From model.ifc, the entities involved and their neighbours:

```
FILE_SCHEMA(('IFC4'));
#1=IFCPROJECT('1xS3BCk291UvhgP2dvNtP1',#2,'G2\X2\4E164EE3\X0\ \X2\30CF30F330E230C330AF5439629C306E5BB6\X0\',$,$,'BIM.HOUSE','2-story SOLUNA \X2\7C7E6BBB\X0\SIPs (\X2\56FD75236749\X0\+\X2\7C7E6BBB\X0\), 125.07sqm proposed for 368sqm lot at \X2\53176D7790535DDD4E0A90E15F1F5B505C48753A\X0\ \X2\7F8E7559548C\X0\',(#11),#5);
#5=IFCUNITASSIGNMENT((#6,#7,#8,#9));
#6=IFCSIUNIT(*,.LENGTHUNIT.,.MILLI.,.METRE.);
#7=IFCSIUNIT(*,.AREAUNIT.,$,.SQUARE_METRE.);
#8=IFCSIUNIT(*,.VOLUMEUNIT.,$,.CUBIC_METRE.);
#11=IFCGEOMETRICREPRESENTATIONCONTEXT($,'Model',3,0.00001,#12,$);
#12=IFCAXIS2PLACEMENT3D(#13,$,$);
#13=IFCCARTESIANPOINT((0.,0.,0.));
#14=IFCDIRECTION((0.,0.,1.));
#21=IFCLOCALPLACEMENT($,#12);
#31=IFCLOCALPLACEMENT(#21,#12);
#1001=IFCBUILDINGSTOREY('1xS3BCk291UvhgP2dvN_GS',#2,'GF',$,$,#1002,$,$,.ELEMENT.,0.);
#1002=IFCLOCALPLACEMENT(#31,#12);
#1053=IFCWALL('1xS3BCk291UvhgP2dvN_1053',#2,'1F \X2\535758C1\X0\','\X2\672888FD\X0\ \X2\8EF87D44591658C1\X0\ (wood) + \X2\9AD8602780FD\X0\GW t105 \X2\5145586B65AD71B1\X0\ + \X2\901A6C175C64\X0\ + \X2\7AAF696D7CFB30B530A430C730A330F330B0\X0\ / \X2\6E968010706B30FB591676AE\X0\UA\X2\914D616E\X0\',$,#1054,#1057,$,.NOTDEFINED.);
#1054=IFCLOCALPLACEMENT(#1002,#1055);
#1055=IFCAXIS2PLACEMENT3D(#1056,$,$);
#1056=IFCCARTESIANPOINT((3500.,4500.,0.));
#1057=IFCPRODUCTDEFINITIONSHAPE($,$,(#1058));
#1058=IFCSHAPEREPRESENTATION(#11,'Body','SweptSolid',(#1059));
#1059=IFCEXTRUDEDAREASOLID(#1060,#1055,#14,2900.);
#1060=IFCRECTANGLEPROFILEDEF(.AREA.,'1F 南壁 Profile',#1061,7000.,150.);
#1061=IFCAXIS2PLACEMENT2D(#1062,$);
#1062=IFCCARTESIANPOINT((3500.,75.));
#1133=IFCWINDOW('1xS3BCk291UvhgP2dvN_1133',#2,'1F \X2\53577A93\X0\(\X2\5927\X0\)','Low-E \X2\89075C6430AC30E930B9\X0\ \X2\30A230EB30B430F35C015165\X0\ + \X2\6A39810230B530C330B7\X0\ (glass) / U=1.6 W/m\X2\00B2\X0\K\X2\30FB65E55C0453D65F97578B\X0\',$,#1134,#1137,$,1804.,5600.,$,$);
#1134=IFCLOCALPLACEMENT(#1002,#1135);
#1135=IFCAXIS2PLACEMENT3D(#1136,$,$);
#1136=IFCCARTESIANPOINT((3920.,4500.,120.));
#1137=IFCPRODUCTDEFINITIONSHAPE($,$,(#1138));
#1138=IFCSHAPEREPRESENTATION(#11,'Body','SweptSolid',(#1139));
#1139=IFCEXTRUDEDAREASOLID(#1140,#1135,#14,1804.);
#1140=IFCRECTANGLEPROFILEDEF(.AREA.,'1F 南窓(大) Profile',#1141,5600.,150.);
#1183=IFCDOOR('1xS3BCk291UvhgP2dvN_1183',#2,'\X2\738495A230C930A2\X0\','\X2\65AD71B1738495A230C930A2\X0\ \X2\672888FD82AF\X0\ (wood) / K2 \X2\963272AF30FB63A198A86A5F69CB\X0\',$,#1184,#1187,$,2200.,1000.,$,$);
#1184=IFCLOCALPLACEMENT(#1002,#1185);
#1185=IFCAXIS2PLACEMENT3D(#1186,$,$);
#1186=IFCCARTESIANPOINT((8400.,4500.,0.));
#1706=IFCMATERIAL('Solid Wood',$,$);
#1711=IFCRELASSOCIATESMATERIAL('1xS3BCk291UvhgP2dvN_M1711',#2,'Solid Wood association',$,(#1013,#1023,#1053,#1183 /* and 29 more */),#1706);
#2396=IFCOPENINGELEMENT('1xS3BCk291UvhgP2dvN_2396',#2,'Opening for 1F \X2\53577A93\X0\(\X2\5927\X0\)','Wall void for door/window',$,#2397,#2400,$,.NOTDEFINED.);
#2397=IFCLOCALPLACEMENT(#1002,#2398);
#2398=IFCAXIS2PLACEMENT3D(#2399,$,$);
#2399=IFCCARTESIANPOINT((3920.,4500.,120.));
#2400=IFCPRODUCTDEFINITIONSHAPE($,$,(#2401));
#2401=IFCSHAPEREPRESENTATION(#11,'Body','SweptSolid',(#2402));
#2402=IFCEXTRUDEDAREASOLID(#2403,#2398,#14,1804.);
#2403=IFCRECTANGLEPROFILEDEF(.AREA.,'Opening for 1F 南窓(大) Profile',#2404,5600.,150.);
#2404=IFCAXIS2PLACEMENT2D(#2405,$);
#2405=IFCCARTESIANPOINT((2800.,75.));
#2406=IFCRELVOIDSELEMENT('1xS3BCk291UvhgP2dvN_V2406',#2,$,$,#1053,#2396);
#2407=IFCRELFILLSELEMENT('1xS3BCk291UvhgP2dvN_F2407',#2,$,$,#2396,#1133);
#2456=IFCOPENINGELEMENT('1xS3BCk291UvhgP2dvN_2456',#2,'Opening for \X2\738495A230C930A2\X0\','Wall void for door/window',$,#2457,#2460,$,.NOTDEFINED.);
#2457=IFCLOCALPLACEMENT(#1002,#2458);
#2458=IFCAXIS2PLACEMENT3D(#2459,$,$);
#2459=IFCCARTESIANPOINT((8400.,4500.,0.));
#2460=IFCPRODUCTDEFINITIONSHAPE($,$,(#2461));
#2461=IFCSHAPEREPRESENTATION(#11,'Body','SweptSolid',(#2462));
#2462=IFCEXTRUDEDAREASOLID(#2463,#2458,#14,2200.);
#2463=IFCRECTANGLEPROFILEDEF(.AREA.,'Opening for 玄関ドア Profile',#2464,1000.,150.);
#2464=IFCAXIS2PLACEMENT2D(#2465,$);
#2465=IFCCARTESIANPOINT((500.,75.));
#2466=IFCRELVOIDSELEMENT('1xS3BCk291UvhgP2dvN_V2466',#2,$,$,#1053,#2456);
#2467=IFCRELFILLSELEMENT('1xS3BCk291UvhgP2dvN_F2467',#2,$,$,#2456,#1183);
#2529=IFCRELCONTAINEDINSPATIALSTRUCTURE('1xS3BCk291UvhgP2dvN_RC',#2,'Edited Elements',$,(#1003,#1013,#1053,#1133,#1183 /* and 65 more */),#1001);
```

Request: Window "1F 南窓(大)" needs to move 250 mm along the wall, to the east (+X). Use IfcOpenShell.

```python
import ifcopenshell
import ifcopenshell.api.geometry
import ifcopenshell.util.placement

model = ifcopenshell.open("model.ifc")

window = model.by_id(1133)
opening = window.FillsVoids[0].RelatingOpeningElement
wall = opening.VoidsElements[0].RelatingBuildingElement

wall_matrix = ifcopenshell.util.placement.get_local_placement(wall.ObjectPlacement)
shift = wall_matrix[:3, 0] * 250.0
before = ifcopenshell.util.placement.get_local_placement(window.ObjectPlacement)[:3, 3].copy()

# The window is not placed relative to its opening, so move both.
for product in (opening, window):
    matrix = ifcopenshell.util.placement.get_local_placement(product.ObjectPlacement)
    matrix[:3, 3] += shift
    ifcopenshell.api.geometry.edit_object_placement(model, product=product, matrix=matrix, is_si=False)

after = ifcopenshell.util.placement.get_local_placement(window.ObjectPlacement)[:3, 3]
print("window moved by", (after - before).round(3) + 0.0)

model.write("model-out.ifc")
```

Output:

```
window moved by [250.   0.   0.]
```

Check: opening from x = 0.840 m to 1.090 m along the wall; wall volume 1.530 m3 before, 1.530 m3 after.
